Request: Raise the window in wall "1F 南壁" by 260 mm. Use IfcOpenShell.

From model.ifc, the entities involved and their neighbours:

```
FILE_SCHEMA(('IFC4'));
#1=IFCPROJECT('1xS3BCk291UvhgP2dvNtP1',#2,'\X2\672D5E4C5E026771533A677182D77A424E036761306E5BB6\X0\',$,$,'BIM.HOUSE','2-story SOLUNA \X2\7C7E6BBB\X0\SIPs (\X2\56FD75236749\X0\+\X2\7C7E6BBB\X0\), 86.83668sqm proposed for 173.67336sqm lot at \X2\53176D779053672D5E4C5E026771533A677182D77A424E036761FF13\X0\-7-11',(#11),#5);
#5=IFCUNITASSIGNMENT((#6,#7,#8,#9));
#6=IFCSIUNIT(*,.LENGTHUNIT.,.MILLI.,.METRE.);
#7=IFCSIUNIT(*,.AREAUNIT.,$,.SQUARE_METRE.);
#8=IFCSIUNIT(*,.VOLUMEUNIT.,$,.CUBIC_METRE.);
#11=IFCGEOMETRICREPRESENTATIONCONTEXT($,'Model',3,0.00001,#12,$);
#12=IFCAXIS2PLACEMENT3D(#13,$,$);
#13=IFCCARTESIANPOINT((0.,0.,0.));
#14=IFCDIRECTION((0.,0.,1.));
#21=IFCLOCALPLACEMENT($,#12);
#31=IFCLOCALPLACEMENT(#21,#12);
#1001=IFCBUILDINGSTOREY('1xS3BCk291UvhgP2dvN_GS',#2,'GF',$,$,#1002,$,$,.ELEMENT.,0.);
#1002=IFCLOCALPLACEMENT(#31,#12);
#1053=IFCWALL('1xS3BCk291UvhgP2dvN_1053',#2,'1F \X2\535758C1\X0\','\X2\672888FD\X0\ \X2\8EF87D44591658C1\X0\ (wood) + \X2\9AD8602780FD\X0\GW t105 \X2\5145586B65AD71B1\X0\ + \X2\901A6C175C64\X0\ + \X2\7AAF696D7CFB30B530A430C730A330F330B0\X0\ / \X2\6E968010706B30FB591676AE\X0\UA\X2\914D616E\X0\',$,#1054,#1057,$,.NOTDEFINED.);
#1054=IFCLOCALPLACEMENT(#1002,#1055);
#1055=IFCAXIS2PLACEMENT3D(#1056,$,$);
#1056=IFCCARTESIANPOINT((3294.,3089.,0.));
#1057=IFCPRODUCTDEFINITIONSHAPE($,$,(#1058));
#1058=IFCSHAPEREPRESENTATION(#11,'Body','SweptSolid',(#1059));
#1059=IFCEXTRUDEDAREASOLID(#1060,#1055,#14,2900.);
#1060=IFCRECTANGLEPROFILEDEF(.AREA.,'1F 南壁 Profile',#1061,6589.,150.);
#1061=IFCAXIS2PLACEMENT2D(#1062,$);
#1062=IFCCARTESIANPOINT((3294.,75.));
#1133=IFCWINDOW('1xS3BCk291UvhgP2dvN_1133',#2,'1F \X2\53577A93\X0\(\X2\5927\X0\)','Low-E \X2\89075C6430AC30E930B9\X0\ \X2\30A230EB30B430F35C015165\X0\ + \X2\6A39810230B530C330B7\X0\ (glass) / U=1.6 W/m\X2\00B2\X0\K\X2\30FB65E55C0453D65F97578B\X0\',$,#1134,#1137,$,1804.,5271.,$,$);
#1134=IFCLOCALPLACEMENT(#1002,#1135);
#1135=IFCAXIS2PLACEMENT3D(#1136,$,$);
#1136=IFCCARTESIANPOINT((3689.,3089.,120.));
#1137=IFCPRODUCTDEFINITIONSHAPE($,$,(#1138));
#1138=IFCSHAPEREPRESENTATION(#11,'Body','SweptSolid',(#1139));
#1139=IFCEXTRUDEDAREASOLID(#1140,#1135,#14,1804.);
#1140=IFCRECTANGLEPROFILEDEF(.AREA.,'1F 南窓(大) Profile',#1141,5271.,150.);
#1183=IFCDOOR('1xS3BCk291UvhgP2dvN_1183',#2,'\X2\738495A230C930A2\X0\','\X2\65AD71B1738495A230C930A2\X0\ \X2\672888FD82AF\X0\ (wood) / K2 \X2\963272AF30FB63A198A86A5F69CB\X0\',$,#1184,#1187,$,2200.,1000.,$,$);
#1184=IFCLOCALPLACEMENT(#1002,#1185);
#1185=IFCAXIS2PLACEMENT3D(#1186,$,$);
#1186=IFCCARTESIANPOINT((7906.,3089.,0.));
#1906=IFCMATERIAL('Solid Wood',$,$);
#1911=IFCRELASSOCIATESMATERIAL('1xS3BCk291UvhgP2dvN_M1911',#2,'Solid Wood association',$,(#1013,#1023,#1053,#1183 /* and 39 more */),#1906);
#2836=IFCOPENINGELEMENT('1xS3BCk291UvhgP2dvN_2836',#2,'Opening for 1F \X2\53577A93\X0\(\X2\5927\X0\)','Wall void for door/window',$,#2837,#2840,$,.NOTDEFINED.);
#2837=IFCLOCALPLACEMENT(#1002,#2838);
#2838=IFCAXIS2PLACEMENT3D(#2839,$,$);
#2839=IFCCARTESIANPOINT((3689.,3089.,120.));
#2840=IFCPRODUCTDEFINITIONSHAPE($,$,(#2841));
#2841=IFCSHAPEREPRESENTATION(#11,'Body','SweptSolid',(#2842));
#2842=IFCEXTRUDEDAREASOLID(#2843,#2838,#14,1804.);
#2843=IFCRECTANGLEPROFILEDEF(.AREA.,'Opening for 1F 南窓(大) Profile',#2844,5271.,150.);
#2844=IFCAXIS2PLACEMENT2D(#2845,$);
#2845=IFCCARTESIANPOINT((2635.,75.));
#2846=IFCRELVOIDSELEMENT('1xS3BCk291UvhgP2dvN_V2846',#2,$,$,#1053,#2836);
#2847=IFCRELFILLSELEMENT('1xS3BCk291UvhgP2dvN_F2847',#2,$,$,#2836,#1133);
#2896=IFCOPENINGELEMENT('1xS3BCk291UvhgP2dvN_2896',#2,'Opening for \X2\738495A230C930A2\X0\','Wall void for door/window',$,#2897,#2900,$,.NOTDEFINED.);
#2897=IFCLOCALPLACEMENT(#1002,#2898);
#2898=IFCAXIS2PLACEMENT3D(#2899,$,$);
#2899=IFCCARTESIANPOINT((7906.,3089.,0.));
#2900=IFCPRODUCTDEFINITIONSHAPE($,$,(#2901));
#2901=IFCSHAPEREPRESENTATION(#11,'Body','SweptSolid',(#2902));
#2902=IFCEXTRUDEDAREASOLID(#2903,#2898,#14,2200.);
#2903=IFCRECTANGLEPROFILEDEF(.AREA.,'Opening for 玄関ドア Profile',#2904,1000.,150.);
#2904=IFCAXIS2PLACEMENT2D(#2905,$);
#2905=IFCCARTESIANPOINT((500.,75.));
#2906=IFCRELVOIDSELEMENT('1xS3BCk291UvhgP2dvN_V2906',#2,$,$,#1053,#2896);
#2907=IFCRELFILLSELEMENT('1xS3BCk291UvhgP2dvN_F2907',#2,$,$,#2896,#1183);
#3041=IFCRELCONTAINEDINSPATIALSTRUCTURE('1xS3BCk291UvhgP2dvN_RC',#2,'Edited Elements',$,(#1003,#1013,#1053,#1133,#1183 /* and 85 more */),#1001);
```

```python
import numpy as np
import ifcopenshell
import ifcopenshell.api.geometry
import ifcopenshell.util.placement
import ifcopenshell.util.unit

model = ifcopenshell.open("model.ifc")
unit_scale = ifcopenshell.util.unit.calculate_unit_scale(model)

window = model.by_guid("1xS3BCk291UvhgP2dvN_1133")
opening = window.FillsVoids[0].RelatingOpeningElement
dz = 0.26 / unit_scale

shift = np.array([0.0, 0.0, dz])
# The window is not placed relative to its opening, so move both.
for product in (opening, window):
    matrix = ifcopenshell.util.placement.get_local_placement(product.ObjectPlacement)
    matrix[:3, 3] += shift
    ifcopenshell.api.geometry.edit_object_placement(model, product=product, matrix=matrix, is_si=False)

print(f"moved by {dz * unit_scale:+.3f} m")

model.write("model-out.ifc")
```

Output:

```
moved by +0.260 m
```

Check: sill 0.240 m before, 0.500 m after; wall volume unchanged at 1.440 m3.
